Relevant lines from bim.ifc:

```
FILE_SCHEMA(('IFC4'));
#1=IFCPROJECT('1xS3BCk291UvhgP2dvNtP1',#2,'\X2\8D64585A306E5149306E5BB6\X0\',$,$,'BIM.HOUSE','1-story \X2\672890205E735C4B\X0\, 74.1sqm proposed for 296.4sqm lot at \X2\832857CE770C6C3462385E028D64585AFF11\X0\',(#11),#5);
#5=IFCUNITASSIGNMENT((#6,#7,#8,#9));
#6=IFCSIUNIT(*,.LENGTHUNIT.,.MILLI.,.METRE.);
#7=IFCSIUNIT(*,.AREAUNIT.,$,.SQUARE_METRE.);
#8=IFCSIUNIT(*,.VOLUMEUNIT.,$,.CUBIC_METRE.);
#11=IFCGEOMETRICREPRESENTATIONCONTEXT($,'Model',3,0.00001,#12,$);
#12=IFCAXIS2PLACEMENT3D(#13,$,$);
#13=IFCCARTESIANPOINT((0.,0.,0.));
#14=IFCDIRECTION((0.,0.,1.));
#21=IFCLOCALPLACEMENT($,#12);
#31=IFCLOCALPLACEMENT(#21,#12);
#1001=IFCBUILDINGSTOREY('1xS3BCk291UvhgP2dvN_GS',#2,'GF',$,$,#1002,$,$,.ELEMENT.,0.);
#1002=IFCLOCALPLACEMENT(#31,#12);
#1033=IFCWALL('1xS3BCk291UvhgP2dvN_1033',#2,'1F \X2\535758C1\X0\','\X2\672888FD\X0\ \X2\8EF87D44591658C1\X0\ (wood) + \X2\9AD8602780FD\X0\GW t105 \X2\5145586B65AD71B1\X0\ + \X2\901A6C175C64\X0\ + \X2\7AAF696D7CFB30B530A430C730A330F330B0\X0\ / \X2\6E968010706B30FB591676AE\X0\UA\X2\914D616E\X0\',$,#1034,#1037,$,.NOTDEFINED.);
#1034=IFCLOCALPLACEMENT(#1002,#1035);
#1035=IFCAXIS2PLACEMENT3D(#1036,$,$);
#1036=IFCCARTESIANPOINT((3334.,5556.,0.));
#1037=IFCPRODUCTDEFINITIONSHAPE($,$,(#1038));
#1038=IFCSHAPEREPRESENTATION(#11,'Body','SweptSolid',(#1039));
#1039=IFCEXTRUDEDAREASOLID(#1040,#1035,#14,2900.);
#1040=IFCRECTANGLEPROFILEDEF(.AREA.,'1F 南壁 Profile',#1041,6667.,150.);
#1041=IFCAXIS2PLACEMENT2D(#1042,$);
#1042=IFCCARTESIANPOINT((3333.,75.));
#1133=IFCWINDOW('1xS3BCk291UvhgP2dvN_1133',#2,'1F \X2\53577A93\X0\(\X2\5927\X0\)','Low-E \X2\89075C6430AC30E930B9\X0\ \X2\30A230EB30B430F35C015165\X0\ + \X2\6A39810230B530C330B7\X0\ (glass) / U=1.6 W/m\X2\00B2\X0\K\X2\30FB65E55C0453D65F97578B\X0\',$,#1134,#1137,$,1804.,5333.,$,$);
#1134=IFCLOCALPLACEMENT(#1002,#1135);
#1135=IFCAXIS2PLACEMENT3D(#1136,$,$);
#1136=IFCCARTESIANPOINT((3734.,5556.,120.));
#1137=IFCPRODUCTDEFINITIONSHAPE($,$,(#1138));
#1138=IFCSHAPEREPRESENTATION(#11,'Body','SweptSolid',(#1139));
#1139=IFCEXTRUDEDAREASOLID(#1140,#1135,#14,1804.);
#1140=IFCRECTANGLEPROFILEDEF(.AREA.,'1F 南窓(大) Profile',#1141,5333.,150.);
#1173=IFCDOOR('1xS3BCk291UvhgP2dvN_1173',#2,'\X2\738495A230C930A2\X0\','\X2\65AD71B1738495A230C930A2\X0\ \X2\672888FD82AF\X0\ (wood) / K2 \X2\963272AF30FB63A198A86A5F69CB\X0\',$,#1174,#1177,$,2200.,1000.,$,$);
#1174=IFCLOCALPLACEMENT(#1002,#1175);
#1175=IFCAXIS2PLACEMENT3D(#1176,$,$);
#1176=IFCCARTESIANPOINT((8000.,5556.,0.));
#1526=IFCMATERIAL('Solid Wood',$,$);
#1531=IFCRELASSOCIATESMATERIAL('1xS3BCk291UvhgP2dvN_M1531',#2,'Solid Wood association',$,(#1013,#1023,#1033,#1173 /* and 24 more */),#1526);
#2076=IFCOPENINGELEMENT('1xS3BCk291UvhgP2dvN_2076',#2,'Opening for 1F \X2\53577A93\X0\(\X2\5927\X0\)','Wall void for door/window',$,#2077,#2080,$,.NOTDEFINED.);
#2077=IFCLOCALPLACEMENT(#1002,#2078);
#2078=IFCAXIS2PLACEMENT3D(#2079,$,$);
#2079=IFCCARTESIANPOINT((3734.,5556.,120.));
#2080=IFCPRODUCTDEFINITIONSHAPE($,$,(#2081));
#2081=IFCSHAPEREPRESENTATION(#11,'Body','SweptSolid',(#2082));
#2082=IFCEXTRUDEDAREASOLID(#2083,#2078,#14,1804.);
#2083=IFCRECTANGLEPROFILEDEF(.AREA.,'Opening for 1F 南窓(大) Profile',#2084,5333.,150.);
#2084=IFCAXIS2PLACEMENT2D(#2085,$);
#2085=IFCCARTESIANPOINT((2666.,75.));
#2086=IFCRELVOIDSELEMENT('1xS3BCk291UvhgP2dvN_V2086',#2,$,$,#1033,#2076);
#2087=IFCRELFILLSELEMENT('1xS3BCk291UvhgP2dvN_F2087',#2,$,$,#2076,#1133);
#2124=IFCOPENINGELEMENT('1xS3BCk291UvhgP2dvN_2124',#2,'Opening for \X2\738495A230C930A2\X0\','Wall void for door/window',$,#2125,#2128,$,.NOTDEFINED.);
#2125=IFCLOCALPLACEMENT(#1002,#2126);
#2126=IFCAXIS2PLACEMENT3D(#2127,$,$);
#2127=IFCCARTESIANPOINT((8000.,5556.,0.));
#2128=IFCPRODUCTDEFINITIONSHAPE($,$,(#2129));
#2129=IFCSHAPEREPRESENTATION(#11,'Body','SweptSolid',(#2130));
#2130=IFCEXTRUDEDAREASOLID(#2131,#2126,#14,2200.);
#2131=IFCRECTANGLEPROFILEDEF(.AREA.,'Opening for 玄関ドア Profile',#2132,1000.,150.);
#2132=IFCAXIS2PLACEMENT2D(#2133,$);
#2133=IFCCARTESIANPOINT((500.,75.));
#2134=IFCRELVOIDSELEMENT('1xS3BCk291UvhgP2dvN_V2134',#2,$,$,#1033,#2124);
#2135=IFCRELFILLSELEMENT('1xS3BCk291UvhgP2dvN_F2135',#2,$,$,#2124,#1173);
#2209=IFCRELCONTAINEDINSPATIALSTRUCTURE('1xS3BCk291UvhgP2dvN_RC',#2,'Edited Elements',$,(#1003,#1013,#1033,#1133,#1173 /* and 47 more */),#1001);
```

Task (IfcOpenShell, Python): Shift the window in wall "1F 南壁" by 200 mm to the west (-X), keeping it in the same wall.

```python
import ifcopenshell
import ifcopenshell.api.geometry
import ifcopenshell.util.placement

model = ifcopenshell.open("bim.ifc")

window = model.by_guid("1xS3BCk291UvhgP2dvN_1133")
opening = window.FillsVoids[0].RelatingOpeningElement
wall = opening.VoidsElements[0].RelatingBuildingElement

wall_matrix = ifcopenshell.util.placement.get_local_placement(wall.ObjectPlacement)
shift = wall_matrix[:3, 0] * -200.0
before = ifcopenshell.util.placement.get_local_placement(window.ObjectPlacement)[:3, 3].copy()

# The window is not placed relative to its opening, so move both.
for product in (opening, window):
    matrix = ifcopenshell.util.placement.get_local_placement(product.ObjectPlacement)
    matrix[:3, 3] += shift
    ifcopenshell.api.geometry.edit_object_placement(model, product=product, matrix=matrix, is_si=False)

after = ifcopenshell.util.placement.get_local_placement(window.ObjectPlacement)[:3, 3]
print("window moved by", (after - before).round(3) + 0.0)

model.write("bim_edited.ifc")
```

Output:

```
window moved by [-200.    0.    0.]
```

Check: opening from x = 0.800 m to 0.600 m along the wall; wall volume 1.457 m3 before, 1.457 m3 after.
